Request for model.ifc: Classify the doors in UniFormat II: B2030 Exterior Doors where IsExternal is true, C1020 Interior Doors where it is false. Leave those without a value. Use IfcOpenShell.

First a look at what the model holds.

```python
import ifcopenshell
import ifcopenshell.util.element

model = ifcopenshell.open("model.ifc")
print(model.schema)
print("classifications:", [c.Name for c in model.by_type("IfcClassification")])
values = [ifcopenshell.util.element.get_pset(e, "Pset_DoorCommon", "IsExternal") for e in model.by_type("IfcDoor")]
for value in (True, False, None):
    print("IsExternal", value, values.count(value))
```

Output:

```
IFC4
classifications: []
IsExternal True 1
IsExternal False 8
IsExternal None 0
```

```python
import ifcopenshell
import ifcopenshell.api.classification
import ifcopenshell.util.element

model = ifcopenshell.open("model.ifc")

system = ifcopenshell.api.classification.add_classification(model, classification="UniFormat II")

doors = model.by_type("IfcDoor")
external = {e: ifcopenshell.util.element.get_pset(e, "Pset_DoorCommon", "IsExternal") for e in doors}
for flag, code, name in ((True, "B2030", "Exterior Doors"), (False, "C1020", "Interior Doors")):
    products = [e for e in doors if external[e] is flag]
    ifcopenshell.api.classification.add_reference(
        model, products=products, classification=system, identification=code, name=name
    )
    print(code, len(products))

model.write("model-out.ifc")
```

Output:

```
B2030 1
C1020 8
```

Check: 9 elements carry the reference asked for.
